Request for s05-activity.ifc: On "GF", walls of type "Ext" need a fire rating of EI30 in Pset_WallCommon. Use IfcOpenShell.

First a look at what the model holds.

```python
import ifcopenshell
import ifcopenshell.util.element

model = ifcopenshell.open("s05-activity.ifc")
print(model.schema)
storey = next(s for s in model.by_type("IfcBuildingStorey") if s.Name == "GF")
walls = [e for e in ifcopenshell.util.element.get_decomposition(storey) if e.is_a("IfcWall")]
seen = {}
for e in walls:
    element_type = ifcopenshell.util.element.get_type(e)
    key = (element_type.Name if element_type != e and element_type else None, ifcopenshell.util.element.get_pset(e, "Pset_WallCommon", "FireRating"))
    seen[key] = seen.get(key, 0) + 1
for (name, value), count in sorted(seen.items(), key=str):
    print(count, "x", name, "|", value)
```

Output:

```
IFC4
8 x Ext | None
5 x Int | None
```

```python
import ifcopenshell
import ifcopenshell.api.pset
import ifcopenshell.util.element

model = ifcopenshell.open("s05-activity.ifc")

storey = next(s for s in model.by_type("IfcBuildingStorey") if s.Name == "GF")
walls = [e for e in ifcopenshell.util.element.get_decomposition(storey) if e.is_a("IfcWall")]

count = 0
for e in walls:
    element_type = ifcopenshell.util.element.get_type(e)
    if element_type in (None, e) or element_type.Name != "Ext":
        continue
    # add_pset returns the element's existing set when there is one.
    pset = ifcopenshell.api.pset.add_pset(model, product=e, name="Pset_WallCommon")
    ifcopenshell.api.pset.edit_pset(model, pset=pset, properties={"FireRating": "EI30"})
    count += 1

print(count, "walls updated")

model.write("s05-activity_v2.ifc")
```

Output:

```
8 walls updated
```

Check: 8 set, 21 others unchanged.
